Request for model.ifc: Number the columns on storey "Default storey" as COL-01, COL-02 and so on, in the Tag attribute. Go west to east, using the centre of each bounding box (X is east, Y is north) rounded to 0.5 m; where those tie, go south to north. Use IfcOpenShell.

First a look at what the model holds.

```python
import ifcopenshell
import ifcopenshell.util.element
import ifcopenshell.util.placement

model = ifcopenshell.open("model.ifc")
print(model.schema)
storey = next(s for s in model.by_type("IfcBuildingStorey") if s.Name == "Default storey")
columns = [e for e in ifcopenshell.util.element.get_decomposition(storey) if e.is_a("IfcColumn")]
for e in sorted(columns, key=lambda e: e.id()):
    origin = ifcopenshell.util.placement.get_local_placement(e.ObjectPlacement)[:3, 3]
    print(e.id(), e.Tag, e.Name, origin.round(2) + 0.0, sep=" | ")
```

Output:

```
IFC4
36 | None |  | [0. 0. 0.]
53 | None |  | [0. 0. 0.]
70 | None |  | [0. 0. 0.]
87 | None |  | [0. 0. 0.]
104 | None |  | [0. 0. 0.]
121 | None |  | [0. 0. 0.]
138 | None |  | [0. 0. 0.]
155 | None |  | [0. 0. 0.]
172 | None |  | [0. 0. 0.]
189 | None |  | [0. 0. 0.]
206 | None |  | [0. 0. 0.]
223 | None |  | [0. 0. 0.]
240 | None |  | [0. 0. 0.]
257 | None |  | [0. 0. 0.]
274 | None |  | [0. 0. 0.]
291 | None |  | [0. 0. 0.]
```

```python
import ifcopenshell
import ifcopenshell.geom
import ifcopenshell.util.element
import ifcopenshell.util.shape

model = ifcopenshell.open("model.ifc")
settings = ifcopenshell.geom.settings()
settings.set("use-world-coords", True)


def centre(element):
    shape = ifcopenshell.geom.create_shape(settings, element)
    return ifcopenshell.util.shape.get_bbox_centroid(shape.geometry)


storey = next(s for s in model.by_type("IfcBuildingStorey") if s.Name == "Default storey")
columns = [e for e in ifcopenshell.util.element.get_decomposition(storey) if e.is_a("IfcColumn")]

# Insertion points can sit at a corner or the storey origin, so sort by the geometry (in metres).
centres = {e: centre(e) for e in columns}
columns.sort(key=lambda e: (round(centres[e][0] / 0.5), centres[e][1]))

for i, e in enumerate(columns, start=1):
    number = f"COL-{i:02d}"
    e.Tag = number
    print(e.id(), number)

model.write("model-out.ifc")
```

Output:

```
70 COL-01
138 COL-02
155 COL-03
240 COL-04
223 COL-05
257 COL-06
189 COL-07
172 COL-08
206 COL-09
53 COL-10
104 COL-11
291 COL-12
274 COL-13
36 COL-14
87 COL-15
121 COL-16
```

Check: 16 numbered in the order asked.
